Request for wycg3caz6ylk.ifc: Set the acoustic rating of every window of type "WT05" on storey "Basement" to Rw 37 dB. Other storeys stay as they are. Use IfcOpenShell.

First a look at what the model holds.

```python
import ifcopenshell
import ifcopenshell.util.element

model = ifcopenshell.open("wycg3caz6ylk.ifc")
print(model.schema)
storey = next(s for s in model.by_type("IfcBuildingStorey") if s.Name == "Basement")
windows = [e for e in ifcopenshell.util.element.get_decomposition(storey) if e.is_a("IfcWindow")]
seen = {}
for e in windows:
    element_type = ifcopenshell.util.element.get_type(e)
    key = (element_type.Name if element_type != e and element_type else None, ifcopenshell.util.element.get_pset(e, "Pset_WindowCommon", "AcousticRating"))
    seen[key] = seen.get(key, 0) + 1
for (name, value), count in sorted(seen.items(), key=str):
    print(count, "x", name, "|", value)
```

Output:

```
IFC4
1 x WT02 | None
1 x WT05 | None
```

```python
import ifcopenshell
import ifcopenshell.api.pset
import ifcopenshell.util.element

model = ifcopenshell.open("wycg3caz6ylk.ifc")

storey = next(s for s in model.by_type("IfcBuildingStorey") if s.Name == "Basement")
windows = [e for e in ifcopenshell.util.element.get_decomposition(storey) if e.is_a("IfcWindow")]

count = 0
for e in windows:
    element_type = ifcopenshell.util.element.get_type(e)
    if element_type in (None, e) or element_type.Name != "WT05":
        continue
    # add_pset returns the element's existing set when there is one.
    pset = ifcopenshell.api.pset.add_pset(model, product=e, name="Pset_WindowCommon")
    ifcopenshell.api.pset.edit_pset(model, pset=pset, properties={"AcousticRating": "Rw 37 dB"})
    count += 1

print(count, "windows updated")

model.write("wycg3caz6ylk_edited.ifc")
```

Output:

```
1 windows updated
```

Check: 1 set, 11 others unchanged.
